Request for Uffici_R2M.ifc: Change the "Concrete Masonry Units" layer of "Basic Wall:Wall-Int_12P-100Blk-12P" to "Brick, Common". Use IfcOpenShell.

First a look at what the model holds.

```python
import ifcopenshell
import ifcopenshell.util.element

model = ifcopenshell.open("Uffici_R2M.ifc")
print(model.schema)
for layer_set in model.by_type("IfcMaterialLayerSet"):
    if layer_set.LayerSetName == "Basic Wall:Wall-Int_12P-100Blk-12P":
        for layer in layer_set.MaterialLayers:
            print(layer.id(), layer.Material and layer.Material.Name, layer.LayerThickness, sep=" | ")
        print(len(ifcopenshell.util.element.get_elements_by_material(model, layer_set)), "elements and types use it")
print(sorted(m.Name for m in model.by_type("IfcMaterial") if m.Name)[:60])
```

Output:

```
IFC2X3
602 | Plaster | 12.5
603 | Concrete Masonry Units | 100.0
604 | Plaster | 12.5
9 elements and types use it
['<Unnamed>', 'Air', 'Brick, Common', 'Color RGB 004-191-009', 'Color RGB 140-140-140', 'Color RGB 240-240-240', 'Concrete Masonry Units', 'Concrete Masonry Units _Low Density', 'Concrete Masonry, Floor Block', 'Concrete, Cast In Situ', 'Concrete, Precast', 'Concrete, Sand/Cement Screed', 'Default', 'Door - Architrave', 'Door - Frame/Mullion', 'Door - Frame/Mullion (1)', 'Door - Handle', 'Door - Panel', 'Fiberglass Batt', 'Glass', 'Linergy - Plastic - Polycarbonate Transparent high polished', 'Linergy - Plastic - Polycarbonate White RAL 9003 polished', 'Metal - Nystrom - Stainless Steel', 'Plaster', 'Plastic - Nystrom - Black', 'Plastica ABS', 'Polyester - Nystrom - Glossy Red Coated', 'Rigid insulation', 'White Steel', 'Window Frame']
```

```python
import ifcopenshell
import ifcopenshell.api.material

model = ifcopenshell.open("Uffici_R2M.ifc")

layer_set = next(s for s in model.by_type("IfcMaterialLayerSet") if s.LayerSetName == "Basic Wall:Wall-Int_12P-100Blk-12P")
layer = next(l for l in layer_set.MaterialLayers if l.Material and l.Material.Name == "Concrete Masonry Units")
material = next(m for m in model.by_type("IfcMaterial") if m.Name == "Brick, Common")

# Point this one layer at the other material; renaming the old one would change it everywhere.
ifcopenshell.api.material.edit_layer(model, layer=layer, attributes={}, material=material)

print([l.Material.Name if l.Material else None for l in layer_set.MaterialLayers])

model.write("Uffici_R2M_edited.ifc")
```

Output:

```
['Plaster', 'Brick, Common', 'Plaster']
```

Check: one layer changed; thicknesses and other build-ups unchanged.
